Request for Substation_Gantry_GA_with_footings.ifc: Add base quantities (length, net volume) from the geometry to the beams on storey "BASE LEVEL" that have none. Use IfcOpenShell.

First a look at what the model holds.

```python
import ifcopenshell
import ifcopenshell.util.element
import ifcopenshell.util.unit

model = ifcopenshell.open("Substation_Gantry_GA_with_footings.ifc")
print(model.schema)
for unit_type in ("LENGTHUNIT", "AREAUNIT", "VOLUMEUNIT"):
    print(unit_type, ifcopenshell.util.unit.calculate_unit_scale(model, unit_type))
storey = next(s for s in model.by_type("IfcBuildingStorey") if s.Name == "BASE LEVEL")
beams = [e for e in ifcopenshell.util.element.get_decomposition(storey) if e.is_a("IfcBeam")]
for e in sorted(beams, key=lambda e: e.id()):
    print(e.id(), e.is_a(), e.Name, list(ifcopenshell.util.element.get_psets(e, qtos_only=True)), sep=" | ")
```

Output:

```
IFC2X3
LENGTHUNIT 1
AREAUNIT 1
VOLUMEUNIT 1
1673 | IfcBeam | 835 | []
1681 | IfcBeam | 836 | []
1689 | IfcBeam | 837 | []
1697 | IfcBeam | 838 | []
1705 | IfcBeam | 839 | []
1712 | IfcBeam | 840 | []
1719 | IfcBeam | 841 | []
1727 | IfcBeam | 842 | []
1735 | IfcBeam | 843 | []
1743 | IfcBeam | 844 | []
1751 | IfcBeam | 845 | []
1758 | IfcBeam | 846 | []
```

```python
import ifcopenshell
import ifcopenshell.api.pset
import ifcopenshell.geom
import ifcopenshell.util.element
import ifcopenshell.util.shape
import ifcopenshell.util.unit

model = ifcopenshell.open("Substation_Gantry_GA_with_footings.ifc")
unit_scale = ifcopenshell.util.unit.calculate_unit_scale(model)
volume_scale = ifcopenshell.util.unit.calculate_unit_scale(model, "VOLUMEUNIT")
settings = ifcopenshell.geom.settings()

storey = next(s for s in model.by_type("IfcBuildingStorey") if s.Name == "BASE LEVEL")
beams = [e for e in ifcopenshell.util.element.get_decomposition(storey) if e.is_a("IfcBeam")]

for e in sorted(beams, key=lambda e: e.id()):
    if ifcopenshell.util.element.get_psets(e, qtos_only=True, should_inherit=False):
        continue
    # Geometry comes back in metres, in the element's own axes.
    shape = ifcopenshell.geom.create_shape(settings, e)
    values = {
        "Length": ifcopenshell.util.shape.get_max_xyz(shape.geometry) / unit_scale,
        "NetVolume": ifcopenshell.util.shape.get_volume(shape.geometry) / volume_scale,
    }
    qto = ifcopenshell.api.pset.add_qto(model, product=e, name="BaseQuantities")
    ifcopenshell.api.pset.edit_qto(model, qto=qto, properties=values)
    print(e.id(), {k: round(v, 3) for k, v in values.items()})

model.write("Substation_Gantry_GA_with_footings_updated.ifc")
```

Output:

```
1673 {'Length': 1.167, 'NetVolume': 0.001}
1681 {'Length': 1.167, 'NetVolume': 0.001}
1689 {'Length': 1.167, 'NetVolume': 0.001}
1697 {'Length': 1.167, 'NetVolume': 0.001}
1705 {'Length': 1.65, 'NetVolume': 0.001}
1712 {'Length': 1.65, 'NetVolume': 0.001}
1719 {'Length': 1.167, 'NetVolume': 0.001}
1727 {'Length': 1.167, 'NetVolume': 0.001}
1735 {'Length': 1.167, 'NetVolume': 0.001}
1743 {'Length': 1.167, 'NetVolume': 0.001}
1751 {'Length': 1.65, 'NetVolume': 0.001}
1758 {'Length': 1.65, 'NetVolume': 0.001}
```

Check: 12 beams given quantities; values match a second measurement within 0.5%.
